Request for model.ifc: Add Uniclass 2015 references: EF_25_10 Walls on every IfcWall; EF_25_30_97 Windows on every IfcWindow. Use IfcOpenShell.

First a look at what the model holds.

```python
import ifcopenshell

model = ifcopenshell.open("model.ifc")
print(model.schema)
print("classifications:", [c.Name for c in model.by_type("IfcClassification")])
for ifc_class in ("IfcDoor", "IfcRoof", "IfcStair", "IfcWall", "IfcWindow"):
    print(ifc_class, len(model.by_type(ifc_class)))
```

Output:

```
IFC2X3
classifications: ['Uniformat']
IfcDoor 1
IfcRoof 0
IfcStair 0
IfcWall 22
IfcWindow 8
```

```python
import ifcopenshell
import ifcopenshell.api.classification

model = ifcopenshell.open("model.ifc")

# IFC2X3 requires Source and Edition and has no link from the project to the system.
system = model.create_entity("IfcClassification", Source="NBS", Edition="2015", Name="Uniclass 2015")

codes = {
    "IfcWall": ("EF_25_10", "Walls"),
    "IfcWindow": ("EF_25_30_97", "Windows"),
}
for ifc_class, (code, name) in codes.items():
    products = model.by_type(ifc_class)
    ifcopenshell.api.classification.add_reference(
        model, products=products, classification=system, identification=code, name=name
    )
    print(code, len(products))

model.write("model-out.ifc")
```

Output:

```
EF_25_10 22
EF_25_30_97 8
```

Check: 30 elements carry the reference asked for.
